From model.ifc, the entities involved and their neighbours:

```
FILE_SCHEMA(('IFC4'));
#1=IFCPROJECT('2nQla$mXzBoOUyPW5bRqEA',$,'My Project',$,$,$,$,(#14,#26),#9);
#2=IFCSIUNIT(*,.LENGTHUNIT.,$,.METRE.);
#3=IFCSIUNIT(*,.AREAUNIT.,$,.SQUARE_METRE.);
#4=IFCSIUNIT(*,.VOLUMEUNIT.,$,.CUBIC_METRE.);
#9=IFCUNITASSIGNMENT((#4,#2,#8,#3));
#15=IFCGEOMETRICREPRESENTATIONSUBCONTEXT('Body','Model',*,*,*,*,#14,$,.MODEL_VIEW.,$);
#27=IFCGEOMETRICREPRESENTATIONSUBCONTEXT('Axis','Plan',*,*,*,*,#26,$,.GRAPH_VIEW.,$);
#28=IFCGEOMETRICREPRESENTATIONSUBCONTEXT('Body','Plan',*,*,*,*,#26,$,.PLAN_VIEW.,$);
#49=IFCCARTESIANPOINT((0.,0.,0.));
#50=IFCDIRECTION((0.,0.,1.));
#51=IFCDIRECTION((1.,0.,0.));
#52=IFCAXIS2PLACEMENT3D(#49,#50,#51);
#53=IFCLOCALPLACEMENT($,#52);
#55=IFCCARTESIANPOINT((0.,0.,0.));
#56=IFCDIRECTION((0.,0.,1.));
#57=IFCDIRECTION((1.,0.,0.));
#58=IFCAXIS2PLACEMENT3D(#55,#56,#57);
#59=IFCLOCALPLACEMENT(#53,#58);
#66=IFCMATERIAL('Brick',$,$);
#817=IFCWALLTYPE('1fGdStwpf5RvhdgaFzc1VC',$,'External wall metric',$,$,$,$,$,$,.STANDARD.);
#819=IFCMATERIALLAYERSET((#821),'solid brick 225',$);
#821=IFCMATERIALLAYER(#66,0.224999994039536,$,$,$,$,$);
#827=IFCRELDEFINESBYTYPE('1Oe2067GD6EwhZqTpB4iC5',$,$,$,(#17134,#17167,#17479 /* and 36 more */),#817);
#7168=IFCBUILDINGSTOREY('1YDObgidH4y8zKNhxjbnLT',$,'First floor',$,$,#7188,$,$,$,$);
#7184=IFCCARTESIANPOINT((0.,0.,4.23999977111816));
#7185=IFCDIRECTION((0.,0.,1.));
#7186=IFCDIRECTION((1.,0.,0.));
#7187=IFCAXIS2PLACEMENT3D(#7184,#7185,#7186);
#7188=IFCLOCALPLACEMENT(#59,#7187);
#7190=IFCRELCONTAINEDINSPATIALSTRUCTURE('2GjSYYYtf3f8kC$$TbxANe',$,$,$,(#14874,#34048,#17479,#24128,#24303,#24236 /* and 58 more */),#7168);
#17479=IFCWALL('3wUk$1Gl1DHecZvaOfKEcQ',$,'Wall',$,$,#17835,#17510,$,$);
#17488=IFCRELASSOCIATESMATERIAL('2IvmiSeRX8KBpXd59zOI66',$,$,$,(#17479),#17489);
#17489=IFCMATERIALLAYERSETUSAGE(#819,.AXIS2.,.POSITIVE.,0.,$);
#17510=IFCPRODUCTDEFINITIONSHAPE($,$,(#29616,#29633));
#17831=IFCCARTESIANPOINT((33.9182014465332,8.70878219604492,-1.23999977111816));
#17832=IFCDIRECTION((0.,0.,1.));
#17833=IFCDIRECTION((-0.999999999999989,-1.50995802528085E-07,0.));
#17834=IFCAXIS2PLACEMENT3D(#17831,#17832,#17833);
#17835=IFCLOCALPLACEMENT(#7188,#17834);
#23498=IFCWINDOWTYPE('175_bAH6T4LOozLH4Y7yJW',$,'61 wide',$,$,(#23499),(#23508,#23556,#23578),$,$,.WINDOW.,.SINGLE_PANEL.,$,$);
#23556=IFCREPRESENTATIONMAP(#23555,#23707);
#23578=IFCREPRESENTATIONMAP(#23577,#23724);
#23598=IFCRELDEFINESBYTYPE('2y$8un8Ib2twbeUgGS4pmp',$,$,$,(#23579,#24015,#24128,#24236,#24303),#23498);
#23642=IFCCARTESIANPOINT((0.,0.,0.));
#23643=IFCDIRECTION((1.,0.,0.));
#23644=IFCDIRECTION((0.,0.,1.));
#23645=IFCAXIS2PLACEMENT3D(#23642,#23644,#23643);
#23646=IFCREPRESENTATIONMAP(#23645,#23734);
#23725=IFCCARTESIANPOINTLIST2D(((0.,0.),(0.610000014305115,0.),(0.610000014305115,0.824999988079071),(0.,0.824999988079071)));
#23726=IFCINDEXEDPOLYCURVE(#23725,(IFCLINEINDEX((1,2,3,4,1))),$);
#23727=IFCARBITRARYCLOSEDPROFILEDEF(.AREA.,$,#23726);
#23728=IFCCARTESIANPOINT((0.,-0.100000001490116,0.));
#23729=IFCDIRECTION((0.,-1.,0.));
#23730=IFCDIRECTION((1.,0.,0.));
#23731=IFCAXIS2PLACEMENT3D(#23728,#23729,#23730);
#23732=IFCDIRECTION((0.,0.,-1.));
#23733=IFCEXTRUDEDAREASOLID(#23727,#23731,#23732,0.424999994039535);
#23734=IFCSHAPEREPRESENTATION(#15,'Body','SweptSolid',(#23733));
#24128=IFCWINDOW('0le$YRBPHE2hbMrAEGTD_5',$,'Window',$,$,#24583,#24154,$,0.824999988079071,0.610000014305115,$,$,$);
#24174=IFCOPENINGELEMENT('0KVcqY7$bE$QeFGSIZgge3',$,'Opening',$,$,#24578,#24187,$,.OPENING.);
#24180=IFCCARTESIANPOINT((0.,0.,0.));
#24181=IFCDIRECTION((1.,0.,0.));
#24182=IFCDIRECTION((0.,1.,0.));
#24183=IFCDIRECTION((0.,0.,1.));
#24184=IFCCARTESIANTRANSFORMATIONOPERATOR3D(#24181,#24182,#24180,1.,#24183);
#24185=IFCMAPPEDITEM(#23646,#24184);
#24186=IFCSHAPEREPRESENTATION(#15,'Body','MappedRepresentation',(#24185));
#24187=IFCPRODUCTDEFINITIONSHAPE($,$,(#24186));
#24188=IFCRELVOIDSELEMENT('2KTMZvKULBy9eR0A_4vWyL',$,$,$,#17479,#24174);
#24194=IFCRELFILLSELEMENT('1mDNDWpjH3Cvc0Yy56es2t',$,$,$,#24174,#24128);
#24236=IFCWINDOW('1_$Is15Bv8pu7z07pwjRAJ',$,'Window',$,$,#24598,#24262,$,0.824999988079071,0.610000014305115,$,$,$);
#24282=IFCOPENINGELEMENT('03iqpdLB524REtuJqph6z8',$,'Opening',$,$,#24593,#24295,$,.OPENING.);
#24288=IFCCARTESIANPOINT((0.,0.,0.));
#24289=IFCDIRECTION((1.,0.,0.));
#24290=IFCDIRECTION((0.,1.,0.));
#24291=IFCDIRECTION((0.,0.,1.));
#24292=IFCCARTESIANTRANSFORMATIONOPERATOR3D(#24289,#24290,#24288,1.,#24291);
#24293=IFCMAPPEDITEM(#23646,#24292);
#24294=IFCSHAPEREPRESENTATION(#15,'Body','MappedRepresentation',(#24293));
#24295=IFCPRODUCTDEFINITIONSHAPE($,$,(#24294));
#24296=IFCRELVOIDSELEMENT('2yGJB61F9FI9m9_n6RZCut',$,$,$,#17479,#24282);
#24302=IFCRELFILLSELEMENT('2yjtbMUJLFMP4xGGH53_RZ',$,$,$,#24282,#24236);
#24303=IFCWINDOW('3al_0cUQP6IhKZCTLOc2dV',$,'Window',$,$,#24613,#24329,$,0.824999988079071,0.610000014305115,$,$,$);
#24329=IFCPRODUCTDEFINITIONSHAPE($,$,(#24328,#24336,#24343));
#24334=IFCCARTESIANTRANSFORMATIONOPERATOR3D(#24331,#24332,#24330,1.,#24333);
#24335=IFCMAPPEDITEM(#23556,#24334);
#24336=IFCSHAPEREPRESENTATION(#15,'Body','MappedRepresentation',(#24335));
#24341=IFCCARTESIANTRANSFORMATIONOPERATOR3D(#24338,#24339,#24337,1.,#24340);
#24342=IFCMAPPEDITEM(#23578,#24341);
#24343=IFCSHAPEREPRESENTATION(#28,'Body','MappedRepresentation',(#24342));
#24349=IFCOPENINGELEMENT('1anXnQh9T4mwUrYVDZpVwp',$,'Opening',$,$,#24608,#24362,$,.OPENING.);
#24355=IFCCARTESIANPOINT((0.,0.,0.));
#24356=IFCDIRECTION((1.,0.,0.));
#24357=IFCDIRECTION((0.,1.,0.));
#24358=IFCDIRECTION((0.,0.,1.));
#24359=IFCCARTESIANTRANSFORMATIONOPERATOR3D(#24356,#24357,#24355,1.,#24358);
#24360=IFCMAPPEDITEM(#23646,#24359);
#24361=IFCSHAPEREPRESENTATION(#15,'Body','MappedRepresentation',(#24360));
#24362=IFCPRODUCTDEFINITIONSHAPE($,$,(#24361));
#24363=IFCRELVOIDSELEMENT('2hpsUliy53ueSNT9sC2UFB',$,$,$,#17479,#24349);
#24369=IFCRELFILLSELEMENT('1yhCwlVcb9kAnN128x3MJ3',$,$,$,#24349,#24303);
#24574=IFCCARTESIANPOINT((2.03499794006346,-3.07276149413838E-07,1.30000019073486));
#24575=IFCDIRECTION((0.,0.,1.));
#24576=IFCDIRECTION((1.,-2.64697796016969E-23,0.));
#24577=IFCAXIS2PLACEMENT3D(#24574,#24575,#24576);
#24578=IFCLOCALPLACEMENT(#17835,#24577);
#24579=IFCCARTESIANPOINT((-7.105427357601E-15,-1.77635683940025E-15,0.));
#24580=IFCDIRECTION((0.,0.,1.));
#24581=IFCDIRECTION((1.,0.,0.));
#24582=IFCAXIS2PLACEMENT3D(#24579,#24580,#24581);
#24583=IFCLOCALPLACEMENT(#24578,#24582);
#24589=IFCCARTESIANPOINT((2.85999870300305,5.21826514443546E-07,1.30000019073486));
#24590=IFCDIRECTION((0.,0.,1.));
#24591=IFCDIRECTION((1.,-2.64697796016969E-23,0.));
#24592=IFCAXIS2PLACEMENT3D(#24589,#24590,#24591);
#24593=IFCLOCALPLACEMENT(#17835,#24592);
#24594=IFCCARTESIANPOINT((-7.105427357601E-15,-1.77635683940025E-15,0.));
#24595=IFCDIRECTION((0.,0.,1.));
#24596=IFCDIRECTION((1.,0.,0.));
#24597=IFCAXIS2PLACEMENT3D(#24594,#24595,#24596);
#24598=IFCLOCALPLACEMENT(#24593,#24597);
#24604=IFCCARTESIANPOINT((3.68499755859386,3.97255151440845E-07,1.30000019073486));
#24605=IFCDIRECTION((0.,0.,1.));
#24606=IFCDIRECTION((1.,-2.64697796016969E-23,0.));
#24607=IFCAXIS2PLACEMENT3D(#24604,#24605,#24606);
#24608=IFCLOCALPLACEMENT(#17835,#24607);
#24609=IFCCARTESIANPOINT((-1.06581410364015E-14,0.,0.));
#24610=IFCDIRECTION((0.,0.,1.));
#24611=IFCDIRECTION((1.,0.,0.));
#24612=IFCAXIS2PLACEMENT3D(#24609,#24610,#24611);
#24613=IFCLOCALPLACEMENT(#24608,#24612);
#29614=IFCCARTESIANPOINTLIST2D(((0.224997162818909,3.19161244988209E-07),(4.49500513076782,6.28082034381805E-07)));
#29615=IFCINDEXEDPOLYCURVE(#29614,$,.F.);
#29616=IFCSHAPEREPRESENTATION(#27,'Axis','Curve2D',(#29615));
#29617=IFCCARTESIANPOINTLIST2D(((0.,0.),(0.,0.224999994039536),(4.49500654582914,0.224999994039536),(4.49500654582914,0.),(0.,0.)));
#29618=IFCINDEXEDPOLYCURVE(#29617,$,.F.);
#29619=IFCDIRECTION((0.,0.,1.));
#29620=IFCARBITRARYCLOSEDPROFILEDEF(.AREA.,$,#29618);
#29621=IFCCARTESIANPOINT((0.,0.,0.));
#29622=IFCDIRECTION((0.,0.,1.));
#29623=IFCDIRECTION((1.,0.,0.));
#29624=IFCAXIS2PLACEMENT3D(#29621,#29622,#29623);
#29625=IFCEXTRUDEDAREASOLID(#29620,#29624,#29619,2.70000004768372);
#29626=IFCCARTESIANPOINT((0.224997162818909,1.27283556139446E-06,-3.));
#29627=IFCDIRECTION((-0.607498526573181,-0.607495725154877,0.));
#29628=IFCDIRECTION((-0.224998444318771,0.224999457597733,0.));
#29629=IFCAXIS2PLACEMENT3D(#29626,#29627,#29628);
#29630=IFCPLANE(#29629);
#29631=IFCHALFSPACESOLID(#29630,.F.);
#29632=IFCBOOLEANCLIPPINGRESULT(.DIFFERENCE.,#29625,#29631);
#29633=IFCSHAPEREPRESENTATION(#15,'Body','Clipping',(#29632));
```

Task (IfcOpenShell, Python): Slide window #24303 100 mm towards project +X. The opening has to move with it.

```python
import ifcopenshell
import ifcopenshell.api.geometry
import ifcopenshell.util.placement

model = ifcopenshell.open("model.ifc")

window = model.by_id(24303)
opening = window.FillsVoids[0].RelatingOpeningElement
wall = opening.VoidsElements[0].RelatingBuildingElement

wall_matrix = ifcopenshell.util.placement.get_local_placement(wall.ObjectPlacement)
shift = wall_matrix[:3, 0] * -0.1
before = ifcopenshell.util.placement.get_local_placement(window.ObjectPlacement)[:3, 3].copy()

# The window is placed relative to its opening, so it follows when the opening moves.
matrix = ifcopenshell.util.placement.get_local_placement(opening.ObjectPlacement)
matrix[:3, 3] += shift
ifcopenshell.api.geometry.edit_object_placement(
    model, product=opening, matrix=matrix, is_si=False, should_transform_children=True
)

after = ifcopenshell.util.placement.get_local_placement(window.ObjectPlacement)[:3, 3]
print("window moved by", (after - before).round(3) + 0.0)

model.write("model-out.ifc")
```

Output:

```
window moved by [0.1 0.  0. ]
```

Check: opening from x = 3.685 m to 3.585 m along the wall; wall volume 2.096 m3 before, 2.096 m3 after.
